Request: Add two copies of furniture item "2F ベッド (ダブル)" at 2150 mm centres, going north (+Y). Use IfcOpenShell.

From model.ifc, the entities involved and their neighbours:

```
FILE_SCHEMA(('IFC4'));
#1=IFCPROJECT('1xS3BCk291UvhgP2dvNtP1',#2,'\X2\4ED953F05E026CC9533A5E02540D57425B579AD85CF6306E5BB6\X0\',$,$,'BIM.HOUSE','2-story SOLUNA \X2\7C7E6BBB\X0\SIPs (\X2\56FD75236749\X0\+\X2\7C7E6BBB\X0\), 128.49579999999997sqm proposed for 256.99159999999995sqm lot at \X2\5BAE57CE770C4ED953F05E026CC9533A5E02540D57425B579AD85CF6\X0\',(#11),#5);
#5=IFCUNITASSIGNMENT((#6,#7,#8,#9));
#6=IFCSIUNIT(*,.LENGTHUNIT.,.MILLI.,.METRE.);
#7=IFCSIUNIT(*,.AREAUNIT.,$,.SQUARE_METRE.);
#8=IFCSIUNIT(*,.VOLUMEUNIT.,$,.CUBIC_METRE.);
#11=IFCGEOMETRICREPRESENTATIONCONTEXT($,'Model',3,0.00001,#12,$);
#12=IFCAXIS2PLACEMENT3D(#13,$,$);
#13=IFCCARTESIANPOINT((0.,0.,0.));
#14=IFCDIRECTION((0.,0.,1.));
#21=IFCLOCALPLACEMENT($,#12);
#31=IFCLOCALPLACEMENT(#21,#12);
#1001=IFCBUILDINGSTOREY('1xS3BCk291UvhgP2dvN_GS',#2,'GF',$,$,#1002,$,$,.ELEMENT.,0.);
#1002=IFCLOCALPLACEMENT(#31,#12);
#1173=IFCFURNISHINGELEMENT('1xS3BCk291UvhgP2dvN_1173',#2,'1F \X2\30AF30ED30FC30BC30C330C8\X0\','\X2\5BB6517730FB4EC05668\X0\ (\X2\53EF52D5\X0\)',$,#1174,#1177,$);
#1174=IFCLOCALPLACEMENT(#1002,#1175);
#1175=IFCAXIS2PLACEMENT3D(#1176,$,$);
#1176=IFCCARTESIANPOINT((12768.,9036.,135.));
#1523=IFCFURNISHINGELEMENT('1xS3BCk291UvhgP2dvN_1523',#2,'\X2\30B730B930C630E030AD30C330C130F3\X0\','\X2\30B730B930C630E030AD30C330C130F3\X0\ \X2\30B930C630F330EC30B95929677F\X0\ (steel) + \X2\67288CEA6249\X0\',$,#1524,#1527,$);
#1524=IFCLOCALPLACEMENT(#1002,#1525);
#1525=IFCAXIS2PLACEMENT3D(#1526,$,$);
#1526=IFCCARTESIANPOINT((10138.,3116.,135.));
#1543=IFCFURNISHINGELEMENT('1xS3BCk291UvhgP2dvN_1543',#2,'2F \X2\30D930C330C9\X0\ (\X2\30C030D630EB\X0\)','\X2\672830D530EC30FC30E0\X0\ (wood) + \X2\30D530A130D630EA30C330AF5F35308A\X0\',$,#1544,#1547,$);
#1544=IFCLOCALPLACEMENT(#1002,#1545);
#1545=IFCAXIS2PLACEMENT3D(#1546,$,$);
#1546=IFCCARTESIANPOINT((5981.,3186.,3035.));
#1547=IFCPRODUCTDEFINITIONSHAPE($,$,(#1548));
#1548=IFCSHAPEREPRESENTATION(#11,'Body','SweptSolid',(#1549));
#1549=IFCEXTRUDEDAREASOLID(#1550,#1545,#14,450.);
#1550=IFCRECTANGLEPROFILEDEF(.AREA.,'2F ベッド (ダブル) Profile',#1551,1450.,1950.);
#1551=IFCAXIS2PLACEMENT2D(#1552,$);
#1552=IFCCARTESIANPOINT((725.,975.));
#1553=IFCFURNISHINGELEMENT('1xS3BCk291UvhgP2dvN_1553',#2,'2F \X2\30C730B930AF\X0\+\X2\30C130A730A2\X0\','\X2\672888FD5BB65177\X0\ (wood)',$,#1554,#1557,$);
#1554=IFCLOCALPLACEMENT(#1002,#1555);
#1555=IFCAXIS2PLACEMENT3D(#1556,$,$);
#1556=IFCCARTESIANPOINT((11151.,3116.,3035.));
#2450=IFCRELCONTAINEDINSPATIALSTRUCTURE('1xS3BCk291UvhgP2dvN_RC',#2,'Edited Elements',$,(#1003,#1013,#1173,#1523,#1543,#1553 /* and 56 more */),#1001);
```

```python
import numpy as np
import ifcopenshell
import ifcopenshell.api.geometry
import ifcopenshell.api.root
import ifcopenshell.util.element
import ifcopenshell.util.placement

model = ifcopenshell.open("model.ifc")


def reuse_history(source, copy):
    """copy_class also copies each property set's owner history, people and application; keep the originals."""
    for rel in copy.IsDefinedBy:
        if rel.is_a("IfcRelDefinesByProperties") and (history := rel.RelatingPropertyDefinition.OwnerHistory):
            rel.RelatingPropertyDefinition.OwnerHistory = source.OwnerHistory
            ifcopenshell.util.element.remove_deep2(model, history)


source = model.by_guid("1xS3BCk291UvhgP2dvN_1543")
base = ifcopenshell.util.placement.get_local_placement(source.ObjectPlacement)
step = np.array([0.0, 1.0, 0.0]) * 2150.0

for i in range(1, 3):
    copy = ifcopenshell.api.root.copy_class(model, product=source)
    copy.Representation = ifcopenshell.util.element.copy_deep(
        model, source.Representation, exclude=["IfcGeometricRepresentationContext", "IfcRepresentationMap"]
    )
    reuse_history(source, copy)
    matrix = base.copy()
    matrix[:3, 3] += i * step
    print("added at", matrix[:3, 3].round(3) + 0.0)
    ifcopenshell.api.geometry.edit_object_placement(model, product=copy, matrix=matrix, is_si=False)

model.write("model-out.ifc")
```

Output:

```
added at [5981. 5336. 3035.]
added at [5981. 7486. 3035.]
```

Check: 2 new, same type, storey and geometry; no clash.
